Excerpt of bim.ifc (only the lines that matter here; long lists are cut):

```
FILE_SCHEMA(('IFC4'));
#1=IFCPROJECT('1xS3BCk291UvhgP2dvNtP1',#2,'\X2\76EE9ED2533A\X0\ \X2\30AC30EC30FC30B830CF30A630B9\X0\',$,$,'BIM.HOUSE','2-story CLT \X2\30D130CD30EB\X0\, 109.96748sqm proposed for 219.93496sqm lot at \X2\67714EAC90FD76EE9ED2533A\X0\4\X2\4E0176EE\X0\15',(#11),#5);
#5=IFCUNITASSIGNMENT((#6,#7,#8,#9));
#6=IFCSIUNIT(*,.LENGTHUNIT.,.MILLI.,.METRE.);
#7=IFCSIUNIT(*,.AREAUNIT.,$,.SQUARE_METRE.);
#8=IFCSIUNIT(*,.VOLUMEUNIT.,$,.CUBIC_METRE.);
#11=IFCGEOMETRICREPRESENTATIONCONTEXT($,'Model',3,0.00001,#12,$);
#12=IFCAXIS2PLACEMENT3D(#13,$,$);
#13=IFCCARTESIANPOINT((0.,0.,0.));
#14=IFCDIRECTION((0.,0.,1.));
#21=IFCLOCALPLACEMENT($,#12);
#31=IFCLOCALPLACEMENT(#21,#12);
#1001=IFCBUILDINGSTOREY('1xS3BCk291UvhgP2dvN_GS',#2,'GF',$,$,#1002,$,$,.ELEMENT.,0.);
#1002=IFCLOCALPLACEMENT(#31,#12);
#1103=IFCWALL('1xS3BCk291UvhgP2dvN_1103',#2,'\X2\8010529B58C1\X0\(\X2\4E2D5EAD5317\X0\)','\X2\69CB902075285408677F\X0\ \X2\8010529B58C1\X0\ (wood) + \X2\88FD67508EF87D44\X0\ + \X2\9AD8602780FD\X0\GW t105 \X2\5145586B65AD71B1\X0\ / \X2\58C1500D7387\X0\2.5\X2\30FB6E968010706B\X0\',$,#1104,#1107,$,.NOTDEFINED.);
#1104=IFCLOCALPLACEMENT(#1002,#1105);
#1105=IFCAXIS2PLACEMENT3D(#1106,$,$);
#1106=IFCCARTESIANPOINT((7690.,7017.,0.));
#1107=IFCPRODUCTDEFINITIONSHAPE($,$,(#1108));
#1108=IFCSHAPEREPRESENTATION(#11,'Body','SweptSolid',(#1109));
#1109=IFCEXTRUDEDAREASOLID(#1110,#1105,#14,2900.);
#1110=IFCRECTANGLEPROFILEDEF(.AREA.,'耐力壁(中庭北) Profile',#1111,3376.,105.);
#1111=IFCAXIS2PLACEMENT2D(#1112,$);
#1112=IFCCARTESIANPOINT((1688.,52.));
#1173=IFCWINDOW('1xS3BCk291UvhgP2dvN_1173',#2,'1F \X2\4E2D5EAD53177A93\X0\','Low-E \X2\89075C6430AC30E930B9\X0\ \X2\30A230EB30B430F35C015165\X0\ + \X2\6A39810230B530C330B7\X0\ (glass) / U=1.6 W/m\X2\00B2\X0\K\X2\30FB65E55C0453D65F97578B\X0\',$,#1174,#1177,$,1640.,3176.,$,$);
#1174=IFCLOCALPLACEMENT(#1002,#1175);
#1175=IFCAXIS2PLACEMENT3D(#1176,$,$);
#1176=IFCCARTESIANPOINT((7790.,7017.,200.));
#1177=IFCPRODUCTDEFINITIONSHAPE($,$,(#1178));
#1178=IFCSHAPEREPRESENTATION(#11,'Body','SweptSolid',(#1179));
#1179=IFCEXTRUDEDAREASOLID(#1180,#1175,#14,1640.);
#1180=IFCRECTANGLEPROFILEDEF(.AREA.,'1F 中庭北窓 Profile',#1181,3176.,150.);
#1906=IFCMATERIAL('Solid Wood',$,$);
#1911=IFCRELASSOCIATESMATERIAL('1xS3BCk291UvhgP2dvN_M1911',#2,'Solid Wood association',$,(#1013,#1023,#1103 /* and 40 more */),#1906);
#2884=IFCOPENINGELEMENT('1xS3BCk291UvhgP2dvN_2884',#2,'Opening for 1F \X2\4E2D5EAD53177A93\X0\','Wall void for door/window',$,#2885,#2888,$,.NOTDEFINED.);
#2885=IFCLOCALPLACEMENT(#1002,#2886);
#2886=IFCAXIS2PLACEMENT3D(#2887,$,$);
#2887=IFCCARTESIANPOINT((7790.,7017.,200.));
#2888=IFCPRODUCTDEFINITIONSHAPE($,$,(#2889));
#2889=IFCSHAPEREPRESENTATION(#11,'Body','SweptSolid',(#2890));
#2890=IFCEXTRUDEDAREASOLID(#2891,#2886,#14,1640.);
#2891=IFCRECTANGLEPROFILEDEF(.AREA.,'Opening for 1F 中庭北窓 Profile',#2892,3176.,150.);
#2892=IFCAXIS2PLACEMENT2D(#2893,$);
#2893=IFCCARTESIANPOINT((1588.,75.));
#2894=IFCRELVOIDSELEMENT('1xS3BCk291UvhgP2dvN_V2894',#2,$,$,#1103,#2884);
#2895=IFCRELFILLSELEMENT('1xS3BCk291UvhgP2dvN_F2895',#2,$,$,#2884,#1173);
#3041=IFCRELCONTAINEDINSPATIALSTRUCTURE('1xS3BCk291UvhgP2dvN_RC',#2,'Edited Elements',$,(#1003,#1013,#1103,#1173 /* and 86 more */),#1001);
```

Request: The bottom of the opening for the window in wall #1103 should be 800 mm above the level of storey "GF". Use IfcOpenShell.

```python
import numpy as np
import ifcopenshell
import ifcopenshell.api.geometry
import ifcopenshell.geom
import ifcopenshell.util.element
import ifcopenshell.util.placement
import ifcopenshell.util.shape
import ifcopenshell.util.unit

model = ifcopenshell.open("bim.ifc")
unit_scale = ifcopenshell.util.unit.calculate_unit_scale(model)

window = model.by_guid("1xS3BCk291UvhgP2dvN_1173")
opening = window.FillsVoids[0].RelatingOpeningElement
storey = ifcopenshell.util.element.get_container(window, ifc_class="IfcBuildingStorey")
level = ifcopenshell.util.placement.get_local_placement(storey.ObjectPlacement)[2, 3]

# The opening's origin need not be at the sill, so measure its lowest point.
shape = ifcopenshell.geom.create_shape(ifcopenshell.geom.settings(), opening)
bottom = ifcopenshell.util.shape.get_shape_bottom_elevation(shape, shape.geometry) / unit_scale
dz = level + 800.0 - bottom

shift = np.array([0.0, 0.0, dz])
# The window is not placed relative to its opening, so move both.
for product in (opening, window):
    matrix = ifcopenshell.util.placement.get_local_placement(product.ObjectPlacement)
    matrix[:3, 3] += shift
    ifcopenshell.api.geometry.edit_object_placement(model, product=product, matrix=matrix, is_si=False)

print(f"moved by {dz * unit_scale:+.3f} m")

model.write("bim_updated.ifc")
```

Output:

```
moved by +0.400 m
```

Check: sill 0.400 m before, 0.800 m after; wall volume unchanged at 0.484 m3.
